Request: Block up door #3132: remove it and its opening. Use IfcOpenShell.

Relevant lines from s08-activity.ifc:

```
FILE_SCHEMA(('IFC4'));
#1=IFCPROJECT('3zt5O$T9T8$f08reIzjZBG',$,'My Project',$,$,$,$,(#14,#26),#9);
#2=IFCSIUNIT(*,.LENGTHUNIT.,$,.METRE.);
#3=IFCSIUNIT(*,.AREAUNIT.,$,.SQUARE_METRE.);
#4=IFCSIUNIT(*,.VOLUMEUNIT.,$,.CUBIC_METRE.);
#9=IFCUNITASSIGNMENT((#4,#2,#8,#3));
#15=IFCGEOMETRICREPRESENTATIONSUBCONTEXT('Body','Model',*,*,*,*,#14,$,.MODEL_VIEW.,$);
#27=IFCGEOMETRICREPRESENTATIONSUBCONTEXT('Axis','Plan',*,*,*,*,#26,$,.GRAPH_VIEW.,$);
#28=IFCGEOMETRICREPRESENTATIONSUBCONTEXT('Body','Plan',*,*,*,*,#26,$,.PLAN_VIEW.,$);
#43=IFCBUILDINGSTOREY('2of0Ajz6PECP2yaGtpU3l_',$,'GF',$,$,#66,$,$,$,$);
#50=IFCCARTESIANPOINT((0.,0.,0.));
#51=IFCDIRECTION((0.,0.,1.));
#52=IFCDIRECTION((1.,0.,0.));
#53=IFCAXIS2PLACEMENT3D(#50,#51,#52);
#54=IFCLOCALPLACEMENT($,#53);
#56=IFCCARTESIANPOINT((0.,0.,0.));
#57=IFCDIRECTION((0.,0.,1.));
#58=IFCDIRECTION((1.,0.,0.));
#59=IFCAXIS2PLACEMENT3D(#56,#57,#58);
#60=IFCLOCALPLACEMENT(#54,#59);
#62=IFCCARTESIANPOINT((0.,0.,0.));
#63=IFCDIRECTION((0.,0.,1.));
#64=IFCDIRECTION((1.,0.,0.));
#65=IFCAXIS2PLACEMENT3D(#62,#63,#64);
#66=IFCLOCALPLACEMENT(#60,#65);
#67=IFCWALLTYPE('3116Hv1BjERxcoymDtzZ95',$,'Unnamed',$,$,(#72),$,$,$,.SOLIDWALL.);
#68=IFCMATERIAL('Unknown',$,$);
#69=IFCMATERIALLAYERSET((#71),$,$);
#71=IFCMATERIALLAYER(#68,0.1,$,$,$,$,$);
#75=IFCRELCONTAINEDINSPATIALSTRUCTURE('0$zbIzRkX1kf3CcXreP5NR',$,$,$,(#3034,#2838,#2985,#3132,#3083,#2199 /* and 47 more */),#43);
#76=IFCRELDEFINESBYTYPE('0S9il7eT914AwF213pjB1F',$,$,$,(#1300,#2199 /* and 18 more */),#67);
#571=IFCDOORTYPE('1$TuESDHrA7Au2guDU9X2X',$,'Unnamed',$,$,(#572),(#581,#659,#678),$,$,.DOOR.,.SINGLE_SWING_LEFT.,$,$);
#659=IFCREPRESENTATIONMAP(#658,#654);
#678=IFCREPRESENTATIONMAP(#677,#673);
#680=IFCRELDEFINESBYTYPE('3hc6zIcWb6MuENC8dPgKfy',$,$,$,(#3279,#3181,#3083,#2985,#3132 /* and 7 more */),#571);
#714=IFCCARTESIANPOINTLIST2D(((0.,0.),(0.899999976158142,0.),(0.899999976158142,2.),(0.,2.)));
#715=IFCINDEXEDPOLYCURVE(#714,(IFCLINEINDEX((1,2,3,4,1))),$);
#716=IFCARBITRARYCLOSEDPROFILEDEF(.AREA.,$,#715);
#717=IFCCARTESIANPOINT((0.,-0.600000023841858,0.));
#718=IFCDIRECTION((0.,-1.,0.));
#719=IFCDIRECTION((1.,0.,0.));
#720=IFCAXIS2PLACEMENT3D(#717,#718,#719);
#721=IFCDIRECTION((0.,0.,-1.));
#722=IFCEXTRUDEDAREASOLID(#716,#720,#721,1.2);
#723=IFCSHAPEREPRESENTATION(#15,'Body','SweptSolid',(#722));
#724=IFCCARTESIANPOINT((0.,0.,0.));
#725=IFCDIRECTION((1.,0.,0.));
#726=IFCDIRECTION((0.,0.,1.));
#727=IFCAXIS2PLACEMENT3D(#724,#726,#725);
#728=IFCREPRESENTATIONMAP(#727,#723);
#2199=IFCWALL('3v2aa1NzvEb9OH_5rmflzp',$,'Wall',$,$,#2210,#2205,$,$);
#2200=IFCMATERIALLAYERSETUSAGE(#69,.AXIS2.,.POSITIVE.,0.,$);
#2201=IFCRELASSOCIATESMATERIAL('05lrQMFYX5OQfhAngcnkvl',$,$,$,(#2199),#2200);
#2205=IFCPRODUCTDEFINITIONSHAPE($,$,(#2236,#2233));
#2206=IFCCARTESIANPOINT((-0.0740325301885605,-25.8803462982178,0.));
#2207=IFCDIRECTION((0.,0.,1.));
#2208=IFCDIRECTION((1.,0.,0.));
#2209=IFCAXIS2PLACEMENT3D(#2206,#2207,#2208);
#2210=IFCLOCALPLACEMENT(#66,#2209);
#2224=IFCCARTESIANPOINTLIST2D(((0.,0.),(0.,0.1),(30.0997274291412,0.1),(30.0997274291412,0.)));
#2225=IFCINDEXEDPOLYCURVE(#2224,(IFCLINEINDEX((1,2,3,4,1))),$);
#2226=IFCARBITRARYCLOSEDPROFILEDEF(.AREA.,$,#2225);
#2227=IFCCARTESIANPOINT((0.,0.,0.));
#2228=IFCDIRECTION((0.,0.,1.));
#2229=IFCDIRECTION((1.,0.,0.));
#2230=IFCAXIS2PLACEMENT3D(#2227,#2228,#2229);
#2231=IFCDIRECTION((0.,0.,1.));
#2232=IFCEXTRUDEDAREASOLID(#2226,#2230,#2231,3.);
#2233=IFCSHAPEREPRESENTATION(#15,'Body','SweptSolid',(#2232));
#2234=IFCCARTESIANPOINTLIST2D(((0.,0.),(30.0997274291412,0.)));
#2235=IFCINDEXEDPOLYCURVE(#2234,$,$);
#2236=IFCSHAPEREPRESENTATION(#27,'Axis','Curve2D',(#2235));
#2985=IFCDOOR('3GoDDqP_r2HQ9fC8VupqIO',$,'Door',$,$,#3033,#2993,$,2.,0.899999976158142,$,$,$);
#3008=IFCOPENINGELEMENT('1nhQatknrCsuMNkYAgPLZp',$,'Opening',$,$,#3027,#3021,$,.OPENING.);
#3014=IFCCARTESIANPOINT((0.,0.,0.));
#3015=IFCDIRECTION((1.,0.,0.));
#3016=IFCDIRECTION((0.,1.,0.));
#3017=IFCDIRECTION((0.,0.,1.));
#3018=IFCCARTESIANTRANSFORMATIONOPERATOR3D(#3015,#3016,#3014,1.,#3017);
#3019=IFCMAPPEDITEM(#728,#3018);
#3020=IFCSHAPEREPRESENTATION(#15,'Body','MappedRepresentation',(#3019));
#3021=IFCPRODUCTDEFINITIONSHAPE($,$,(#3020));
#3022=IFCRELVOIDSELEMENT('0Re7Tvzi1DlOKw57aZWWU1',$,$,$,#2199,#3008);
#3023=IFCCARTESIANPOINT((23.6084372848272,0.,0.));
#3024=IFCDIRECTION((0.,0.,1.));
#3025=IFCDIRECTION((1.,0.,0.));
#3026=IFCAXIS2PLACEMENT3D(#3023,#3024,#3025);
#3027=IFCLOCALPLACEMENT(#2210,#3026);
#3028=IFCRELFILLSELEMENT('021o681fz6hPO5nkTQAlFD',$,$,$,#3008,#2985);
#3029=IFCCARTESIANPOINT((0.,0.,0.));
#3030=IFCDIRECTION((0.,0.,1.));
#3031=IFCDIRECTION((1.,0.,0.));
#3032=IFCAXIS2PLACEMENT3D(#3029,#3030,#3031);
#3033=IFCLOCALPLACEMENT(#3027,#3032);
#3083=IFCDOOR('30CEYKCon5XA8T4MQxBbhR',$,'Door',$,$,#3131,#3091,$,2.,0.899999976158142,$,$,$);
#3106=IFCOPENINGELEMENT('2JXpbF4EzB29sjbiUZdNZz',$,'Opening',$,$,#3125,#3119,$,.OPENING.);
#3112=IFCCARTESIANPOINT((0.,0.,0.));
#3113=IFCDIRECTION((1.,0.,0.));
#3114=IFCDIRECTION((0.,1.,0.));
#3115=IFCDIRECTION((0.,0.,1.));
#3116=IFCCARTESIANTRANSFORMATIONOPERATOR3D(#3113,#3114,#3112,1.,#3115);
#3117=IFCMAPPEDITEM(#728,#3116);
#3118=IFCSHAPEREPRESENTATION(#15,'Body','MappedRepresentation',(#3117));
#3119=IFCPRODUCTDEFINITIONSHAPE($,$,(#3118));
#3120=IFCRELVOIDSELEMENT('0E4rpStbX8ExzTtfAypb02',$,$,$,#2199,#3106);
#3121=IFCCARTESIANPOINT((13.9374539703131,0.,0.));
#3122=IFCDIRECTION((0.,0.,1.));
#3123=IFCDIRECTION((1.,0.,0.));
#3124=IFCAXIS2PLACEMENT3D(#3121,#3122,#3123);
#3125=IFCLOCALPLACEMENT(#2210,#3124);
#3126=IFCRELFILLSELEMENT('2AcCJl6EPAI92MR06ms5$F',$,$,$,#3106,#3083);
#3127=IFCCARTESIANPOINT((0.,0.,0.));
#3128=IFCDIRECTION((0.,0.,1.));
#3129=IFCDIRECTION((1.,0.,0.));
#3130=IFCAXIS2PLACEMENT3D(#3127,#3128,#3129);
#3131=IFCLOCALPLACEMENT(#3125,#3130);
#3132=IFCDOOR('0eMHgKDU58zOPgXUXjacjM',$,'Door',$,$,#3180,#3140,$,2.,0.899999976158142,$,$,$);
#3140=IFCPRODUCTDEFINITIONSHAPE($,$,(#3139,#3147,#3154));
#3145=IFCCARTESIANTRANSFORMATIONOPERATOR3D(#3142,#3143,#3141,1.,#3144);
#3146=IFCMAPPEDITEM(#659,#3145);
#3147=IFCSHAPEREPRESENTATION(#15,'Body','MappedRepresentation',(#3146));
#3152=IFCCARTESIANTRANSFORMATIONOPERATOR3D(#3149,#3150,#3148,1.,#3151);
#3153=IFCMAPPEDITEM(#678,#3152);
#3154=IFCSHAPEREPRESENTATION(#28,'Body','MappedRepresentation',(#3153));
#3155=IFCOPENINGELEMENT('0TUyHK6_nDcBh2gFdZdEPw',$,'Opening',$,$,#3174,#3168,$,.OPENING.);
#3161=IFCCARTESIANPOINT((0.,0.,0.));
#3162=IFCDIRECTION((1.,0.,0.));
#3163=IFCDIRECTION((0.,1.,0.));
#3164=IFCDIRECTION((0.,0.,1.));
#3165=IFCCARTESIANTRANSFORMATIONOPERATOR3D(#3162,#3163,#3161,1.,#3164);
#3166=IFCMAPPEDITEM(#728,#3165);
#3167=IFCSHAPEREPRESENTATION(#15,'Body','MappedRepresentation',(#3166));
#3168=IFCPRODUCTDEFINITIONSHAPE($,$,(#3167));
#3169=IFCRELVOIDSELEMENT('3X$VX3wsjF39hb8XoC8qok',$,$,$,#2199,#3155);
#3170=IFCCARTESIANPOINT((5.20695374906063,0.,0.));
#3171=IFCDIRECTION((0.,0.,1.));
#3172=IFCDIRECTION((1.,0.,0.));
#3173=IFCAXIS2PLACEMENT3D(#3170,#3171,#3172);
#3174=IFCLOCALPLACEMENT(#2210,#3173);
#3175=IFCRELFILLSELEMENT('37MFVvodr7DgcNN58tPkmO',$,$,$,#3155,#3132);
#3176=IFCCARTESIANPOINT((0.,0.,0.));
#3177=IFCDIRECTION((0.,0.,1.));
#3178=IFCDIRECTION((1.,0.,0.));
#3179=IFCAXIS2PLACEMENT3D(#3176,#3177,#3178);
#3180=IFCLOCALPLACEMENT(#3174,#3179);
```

```python
import ifcopenshell
import ifcopenshell.api.feature
import ifcopenshell.api.root
import ifcopenshell.geom
import ifcopenshell.util.shape

model = ifcopenshell.open("s08-activity.ifc")
settings = ifcopenshell.geom.settings()


def volume(element):
    """Net volume in cubic metres, openings subtracted."""
    shape = ifcopenshell.geom.create_shape(settings, element)
    return ifcopenshell.util.shape.get_volume(shape.geometry)


door = model.by_guid("0eMHgKDU58zOPgXUXjacjM")
opening = door.FillsVoids[0].RelatingOpeningElement
wall = opening.VoidsElements[0].RelatingBuildingElement
before = volume(wall)

ifcopenshell.api.root.remove_product(model, product=door)
ifcopenshell.api.feature.remove_feature(model, feature=opening)

after = volume(wall)

print(f"wall volume {before:.3f} -> {after:.3f} m3")

model.write("s08-activity-out.ifc")
```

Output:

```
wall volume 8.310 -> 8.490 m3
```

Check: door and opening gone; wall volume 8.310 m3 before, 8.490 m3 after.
